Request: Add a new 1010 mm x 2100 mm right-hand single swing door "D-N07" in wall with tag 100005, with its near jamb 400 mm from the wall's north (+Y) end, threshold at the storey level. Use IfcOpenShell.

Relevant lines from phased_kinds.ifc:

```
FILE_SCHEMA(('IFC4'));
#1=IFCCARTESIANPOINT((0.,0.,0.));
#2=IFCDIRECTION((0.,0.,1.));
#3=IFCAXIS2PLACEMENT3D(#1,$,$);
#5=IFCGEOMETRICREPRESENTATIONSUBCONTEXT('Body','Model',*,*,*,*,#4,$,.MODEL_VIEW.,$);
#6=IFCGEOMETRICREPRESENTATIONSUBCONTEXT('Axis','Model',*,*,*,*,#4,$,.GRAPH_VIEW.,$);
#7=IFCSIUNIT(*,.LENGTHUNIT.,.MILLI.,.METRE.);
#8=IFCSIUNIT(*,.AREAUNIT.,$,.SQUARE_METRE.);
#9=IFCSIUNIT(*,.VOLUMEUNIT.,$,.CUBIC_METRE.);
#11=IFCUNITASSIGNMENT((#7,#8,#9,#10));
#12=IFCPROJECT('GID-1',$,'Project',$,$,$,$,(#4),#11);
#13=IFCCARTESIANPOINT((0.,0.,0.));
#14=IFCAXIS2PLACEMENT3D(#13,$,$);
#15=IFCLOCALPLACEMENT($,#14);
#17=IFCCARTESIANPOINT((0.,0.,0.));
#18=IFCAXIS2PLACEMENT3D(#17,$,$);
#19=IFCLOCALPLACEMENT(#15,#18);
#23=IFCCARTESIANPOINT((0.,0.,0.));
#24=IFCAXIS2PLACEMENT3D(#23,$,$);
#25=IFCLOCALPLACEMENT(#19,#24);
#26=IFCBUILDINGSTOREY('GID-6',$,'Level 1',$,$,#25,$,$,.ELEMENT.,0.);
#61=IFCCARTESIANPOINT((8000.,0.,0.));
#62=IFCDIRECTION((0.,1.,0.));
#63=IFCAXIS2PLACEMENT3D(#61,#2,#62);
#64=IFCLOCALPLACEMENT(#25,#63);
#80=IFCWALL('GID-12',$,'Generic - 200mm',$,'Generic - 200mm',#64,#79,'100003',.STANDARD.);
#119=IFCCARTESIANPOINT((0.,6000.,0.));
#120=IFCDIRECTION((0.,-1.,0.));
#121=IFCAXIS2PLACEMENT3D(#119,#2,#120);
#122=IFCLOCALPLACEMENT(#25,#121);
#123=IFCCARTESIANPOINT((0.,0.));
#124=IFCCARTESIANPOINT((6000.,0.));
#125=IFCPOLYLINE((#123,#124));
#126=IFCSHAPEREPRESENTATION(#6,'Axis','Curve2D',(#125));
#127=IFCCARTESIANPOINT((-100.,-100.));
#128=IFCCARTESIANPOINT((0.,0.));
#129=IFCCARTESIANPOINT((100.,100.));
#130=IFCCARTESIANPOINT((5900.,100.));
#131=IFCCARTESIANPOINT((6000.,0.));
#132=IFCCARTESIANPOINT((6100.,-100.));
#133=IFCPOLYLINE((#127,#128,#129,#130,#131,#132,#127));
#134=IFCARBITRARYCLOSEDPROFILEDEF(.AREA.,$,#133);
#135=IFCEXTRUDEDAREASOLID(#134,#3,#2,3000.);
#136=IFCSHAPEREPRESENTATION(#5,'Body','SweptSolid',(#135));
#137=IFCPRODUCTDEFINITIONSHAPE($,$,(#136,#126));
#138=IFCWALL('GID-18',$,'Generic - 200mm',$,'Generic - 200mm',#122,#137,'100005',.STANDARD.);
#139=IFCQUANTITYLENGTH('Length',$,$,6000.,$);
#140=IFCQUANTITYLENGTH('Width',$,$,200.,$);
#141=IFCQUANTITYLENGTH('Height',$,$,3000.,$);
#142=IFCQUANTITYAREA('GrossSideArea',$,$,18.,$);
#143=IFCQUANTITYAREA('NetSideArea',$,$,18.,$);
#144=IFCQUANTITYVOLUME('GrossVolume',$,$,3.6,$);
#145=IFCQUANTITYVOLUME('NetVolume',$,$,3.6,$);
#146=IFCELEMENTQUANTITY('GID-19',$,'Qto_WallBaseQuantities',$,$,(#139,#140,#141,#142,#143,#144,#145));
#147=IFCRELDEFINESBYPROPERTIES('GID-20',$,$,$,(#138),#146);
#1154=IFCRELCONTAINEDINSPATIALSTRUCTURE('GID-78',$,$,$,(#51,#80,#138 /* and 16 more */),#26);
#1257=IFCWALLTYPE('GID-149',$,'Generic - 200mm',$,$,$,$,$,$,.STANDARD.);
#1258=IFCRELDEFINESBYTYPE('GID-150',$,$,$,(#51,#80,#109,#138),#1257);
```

```python
import numpy as np
import ifcopenshell
import ifcopenshell.api.feature
import ifcopenshell.api.geometry
import ifcopenshell.api.pset
import ifcopenshell.api.root
import ifcopenshell.api.spatial
import ifcopenshell.geom
import ifcopenshell.util.element
import ifcopenshell.util.placement
import ifcopenshell.util.representation
import ifcopenshell.util.shape
import ifcopenshell.util.unit

model = ifcopenshell.open("phased_kinds.ifc")
unit_scale = ifcopenshell.util.unit.calculate_unit_scale(model)
area_scale = ifcopenshell.util.unit.calculate_unit_scale(model, "AREAUNIT")
volume_scale = ifcopenshell.util.unit.calculate_unit_scale(model, "VOLUMEUNIT")
settings = ifcopenshell.geom.settings()


def volume(element):
    """Net volume in cubic metres, openings subtracted."""
    shape = ifcopenshell.geom.create_shape(settings, element)
    return ifcopenshell.util.shape.get_volume(shape.geometry)


wall = model.by_guid("GID-18")
storey = ifcopenshell.util.element.get_container(wall, ifc_class="IfcBuildingStorey")
context = ifcopenshell.util.representation.get_context(model, "Model", "Body", "MODEL_VIEW")
before = volume(wall)

width, height, from_end, sill = 1.01, 2.1, 0.4, 0.0  # metres

# The wall runs along its own X axis, and the end named is its -X end.
wall_shape = ifcopenshell.geom.create_shape(settings, wall)
x, y, z = ifcopenshell.util.shape.get_vertices(wall_shape.geometry).T
start = x.min() + from_end
face, thickness = float(y.min()), float(y.max() - y.min())
wall_matrix = ifcopenshell.util.placement.get_local_placement(wall.ObjectPlacement)
level = ifcopenshell.util.placement.get_local_placement(storey.ObjectPlacement)[2, 3]


def in_wall(x, y):
    """Placement at x, y metres in the wall's axes, at sill height."""
    matrix = wall_matrix.copy()
    matrix[:, 3] = wall_matrix @ np.array([x / unit_scale, y / unit_scale, 0.0, 1.0])
    matrix[2, 3] = level + sill / unit_scale
    return matrix


# Opening: a box that overshoots both wall faces by 50 mm.
opening = ifcopenshell.api.root.create_entity(model, ifc_class="IfcOpeningElement", predefined_type="OPENING")
box = ifcopenshell.api.geometry.add_wall_representation(
    model, context=context, length=width, height=height, thickness=thickness + 0.1
)
ifcopenshell.api.geometry.assign_representation(model, product=opening, representation=box)
ifcopenshell.api.geometry.edit_object_placement(model, product=opening, matrix=in_wall(start, face - 0.05), is_si=False)
ifcopenshell.api.feature.add_feature(model, feature=opening, element=wall)

door = ifcopenshell.api.root.create_entity(model, ifc_class="IfcDoor", name="D-N07", predefined_type="DOOR")
door.OverallWidth, door.OverallHeight = width / unit_scale, height / unit_scale
door.OperationType = "SINGLE_SWING_RIGHT"
body = ifcopenshell.api.geometry.add_door_representation(
    model,
    context=context,
    overall_width=door.OverallWidth,
    overall_height=door.OverallHeight,
    operation_type="SINGLE_SWING_RIGHT",
    lining_properties={"LiningDepth": thickness / unit_scale, "ThresholdDepth": thickness / unit_scale},
)
ifcopenshell.api.geometry.assign_representation(model, product=door, representation=body)
ifcopenshell.api.spatial.assign_container(model, products=[door], relating_structure=storey)
ifcopenshell.api.feature.add_filling(model, opening=opening, element=door)

# The lining spans the wall, so the door starts at the wall face.
ifcopenshell.api.geometry.edit_object_placement(model, product=door, matrix=in_wall(start, face), is_si=False)

after = volume(wall)

# Update the wall's stored quantities.
qto = model.by_id(ifcopenshell.util.element.get_pset(wall, "Qto_WallBaseQuantities", should_inherit=False)["id"])
ifcopenshell.api.pset.edit_qto(model, qto=qto, properties={
    "NetSideArea": after / thickness / area_scale,
    "NetVolume": after / volume_scale,
})

print(f"wall volume {before:.3f} -> {after:.3f} m3")

model.write("phased_kinds_updated.ifc")
```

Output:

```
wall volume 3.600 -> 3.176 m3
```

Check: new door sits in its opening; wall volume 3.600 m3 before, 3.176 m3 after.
